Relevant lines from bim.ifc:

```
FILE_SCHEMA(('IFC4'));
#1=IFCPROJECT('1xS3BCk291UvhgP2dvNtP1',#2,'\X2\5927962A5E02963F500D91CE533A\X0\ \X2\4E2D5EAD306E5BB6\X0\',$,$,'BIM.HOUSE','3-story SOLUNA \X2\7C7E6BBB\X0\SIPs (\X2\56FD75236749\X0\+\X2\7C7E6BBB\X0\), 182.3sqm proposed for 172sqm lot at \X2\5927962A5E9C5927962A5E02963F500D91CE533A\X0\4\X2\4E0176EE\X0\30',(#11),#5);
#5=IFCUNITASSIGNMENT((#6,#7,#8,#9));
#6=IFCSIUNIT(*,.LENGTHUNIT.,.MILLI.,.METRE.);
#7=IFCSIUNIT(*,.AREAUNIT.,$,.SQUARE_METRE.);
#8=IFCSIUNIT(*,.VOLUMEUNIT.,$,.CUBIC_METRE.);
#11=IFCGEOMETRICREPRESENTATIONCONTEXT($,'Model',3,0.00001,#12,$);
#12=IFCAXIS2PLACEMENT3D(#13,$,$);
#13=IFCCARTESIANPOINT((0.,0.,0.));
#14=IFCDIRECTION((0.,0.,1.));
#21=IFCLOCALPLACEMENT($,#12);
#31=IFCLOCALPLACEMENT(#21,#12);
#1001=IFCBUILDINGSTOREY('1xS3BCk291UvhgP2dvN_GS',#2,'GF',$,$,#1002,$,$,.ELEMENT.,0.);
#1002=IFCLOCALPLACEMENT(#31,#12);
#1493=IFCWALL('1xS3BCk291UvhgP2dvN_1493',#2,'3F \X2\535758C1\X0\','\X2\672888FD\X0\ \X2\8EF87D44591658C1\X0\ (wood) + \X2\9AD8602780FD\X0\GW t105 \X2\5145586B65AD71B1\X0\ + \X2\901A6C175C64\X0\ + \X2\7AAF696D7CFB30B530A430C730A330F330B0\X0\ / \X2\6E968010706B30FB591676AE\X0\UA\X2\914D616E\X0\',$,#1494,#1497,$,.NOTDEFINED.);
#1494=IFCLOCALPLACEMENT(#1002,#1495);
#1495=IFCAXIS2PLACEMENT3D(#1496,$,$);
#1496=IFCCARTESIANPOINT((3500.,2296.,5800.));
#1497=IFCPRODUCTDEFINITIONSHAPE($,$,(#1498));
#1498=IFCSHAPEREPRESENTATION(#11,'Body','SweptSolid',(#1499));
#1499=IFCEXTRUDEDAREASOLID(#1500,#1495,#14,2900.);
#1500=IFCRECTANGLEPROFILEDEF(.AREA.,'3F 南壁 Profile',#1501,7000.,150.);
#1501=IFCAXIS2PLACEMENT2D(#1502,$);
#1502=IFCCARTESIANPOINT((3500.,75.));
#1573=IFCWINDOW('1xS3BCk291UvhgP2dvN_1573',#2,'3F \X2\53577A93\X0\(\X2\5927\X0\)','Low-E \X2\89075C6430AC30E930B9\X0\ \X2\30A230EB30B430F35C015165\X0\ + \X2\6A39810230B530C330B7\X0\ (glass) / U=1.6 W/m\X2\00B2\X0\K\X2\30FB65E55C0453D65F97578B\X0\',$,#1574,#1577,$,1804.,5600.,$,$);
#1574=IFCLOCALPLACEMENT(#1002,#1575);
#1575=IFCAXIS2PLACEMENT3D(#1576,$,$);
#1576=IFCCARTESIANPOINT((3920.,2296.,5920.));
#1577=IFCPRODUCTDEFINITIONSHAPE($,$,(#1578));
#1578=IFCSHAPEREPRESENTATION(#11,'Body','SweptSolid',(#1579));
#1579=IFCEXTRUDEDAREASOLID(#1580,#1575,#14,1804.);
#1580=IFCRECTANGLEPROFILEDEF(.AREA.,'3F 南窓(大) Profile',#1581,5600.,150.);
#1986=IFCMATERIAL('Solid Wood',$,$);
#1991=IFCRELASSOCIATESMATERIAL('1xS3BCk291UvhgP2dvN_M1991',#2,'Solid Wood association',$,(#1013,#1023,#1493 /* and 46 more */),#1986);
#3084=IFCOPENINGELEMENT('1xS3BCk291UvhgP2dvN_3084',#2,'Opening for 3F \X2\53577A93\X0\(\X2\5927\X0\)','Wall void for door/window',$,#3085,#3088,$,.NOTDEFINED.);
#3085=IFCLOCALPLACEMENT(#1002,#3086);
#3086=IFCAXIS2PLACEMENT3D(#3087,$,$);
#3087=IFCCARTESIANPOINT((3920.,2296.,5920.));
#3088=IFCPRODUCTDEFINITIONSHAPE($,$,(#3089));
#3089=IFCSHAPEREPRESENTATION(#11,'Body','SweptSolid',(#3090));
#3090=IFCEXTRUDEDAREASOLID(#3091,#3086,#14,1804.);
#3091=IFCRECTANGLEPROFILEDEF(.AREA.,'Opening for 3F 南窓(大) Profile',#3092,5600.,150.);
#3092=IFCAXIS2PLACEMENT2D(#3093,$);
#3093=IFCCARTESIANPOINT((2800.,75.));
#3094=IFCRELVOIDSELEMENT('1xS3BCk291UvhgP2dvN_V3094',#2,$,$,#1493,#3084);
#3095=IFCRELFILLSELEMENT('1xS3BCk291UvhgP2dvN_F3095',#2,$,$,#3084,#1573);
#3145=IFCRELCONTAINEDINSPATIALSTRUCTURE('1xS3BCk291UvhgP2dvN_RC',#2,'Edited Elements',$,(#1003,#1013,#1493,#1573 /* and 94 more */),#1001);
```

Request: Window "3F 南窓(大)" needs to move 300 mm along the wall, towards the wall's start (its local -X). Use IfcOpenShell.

```python
import ifcopenshell
import ifcopenshell.api.geometry
import ifcopenshell.util.placement
import ifcopenshell.util.unit

model = ifcopenshell.open("bim.ifc")
unit_scale = ifcopenshell.util.unit.calculate_unit_scale(model)

window = model.by_guid("1xS3BCk291UvhgP2dvN_1573")
opening = window.FillsVoids[0].RelatingOpeningElement
wall = opening.VoidsElements[0].RelatingBuildingElement

wall_matrix = ifcopenshell.util.placement.get_local_placement(wall.ObjectPlacement)
shift = wall_matrix[:3, 0] * -0.3 / unit_scale
before = ifcopenshell.util.placement.get_local_placement(window.ObjectPlacement)[:3, 3].copy()

# The window is not placed relative to its opening, so move both.
for product in (opening, window):
    matrix = ifcopenshell.util.placement.get_local_placement(product.ObjectPlacement)
    matrix[:3, 3] += shift
    ifcopenshell.api.geometry.edit_object_placement(model, product=product, matrix=matrix, is_si=False)

after = ifcopenshell.util.placement.get_local_placement(window.ObjectPlacement)[:3, 3]
print("window moved by", (after - before).round(3) + 0.0)

model.write("bim_rev.ifc")
```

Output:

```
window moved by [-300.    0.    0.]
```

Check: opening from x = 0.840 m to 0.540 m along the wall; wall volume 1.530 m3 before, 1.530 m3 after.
